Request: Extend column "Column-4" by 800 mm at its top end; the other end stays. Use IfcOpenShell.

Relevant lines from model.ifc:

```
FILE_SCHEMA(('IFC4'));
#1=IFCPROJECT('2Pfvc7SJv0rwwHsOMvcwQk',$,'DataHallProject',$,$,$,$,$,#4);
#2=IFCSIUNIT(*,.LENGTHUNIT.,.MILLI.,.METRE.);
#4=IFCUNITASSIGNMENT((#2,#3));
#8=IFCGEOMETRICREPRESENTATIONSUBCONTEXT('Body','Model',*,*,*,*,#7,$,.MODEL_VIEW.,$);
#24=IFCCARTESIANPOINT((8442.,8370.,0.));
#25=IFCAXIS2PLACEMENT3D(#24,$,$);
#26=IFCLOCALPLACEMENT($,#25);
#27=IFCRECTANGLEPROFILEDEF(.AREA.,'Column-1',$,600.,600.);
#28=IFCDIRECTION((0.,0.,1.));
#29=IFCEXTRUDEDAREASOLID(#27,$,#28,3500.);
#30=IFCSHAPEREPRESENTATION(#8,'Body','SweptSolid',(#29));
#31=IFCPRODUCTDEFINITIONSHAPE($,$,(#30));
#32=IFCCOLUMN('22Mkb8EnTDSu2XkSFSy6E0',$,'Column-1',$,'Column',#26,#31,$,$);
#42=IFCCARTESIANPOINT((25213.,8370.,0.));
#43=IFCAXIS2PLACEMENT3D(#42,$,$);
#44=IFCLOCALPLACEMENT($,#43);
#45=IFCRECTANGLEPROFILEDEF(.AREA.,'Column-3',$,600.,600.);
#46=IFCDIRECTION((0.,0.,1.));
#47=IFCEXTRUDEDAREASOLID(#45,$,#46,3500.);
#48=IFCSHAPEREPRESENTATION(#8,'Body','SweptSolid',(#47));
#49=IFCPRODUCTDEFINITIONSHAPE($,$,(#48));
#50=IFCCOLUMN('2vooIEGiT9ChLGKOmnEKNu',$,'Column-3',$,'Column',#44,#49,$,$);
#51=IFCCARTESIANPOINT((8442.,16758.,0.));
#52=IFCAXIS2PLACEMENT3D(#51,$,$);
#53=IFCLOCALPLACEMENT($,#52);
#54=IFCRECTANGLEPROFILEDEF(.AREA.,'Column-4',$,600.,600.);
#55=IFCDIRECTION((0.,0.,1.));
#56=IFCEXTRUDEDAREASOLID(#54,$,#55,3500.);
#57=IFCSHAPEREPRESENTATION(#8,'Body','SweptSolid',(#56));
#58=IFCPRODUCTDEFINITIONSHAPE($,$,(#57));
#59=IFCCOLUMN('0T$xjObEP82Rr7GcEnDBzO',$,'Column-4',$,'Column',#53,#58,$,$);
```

```python
import ifcopenshell
import ifcopenshell.util.representation
import ifcopenshell.util.unit

model = ifcopenshell.open("model.ifc")
unit_scale = ifcopenshell.util.unit.calculate_unit_scale(model)

member = model.by_guid("0T$xjObEP82Rr7GcEnDBzO")
change = 0.8 / unit_scale

# The extrusion runs towards the end named, so only its depth changes.
body = ifcopenshell.util.representation.get_representation(member, "Model", "Body")
solid = body.Items[0]
old_length = solid.Depth
solid.Depth += change

print(f"length {old_length:g} -> {solid.Depth:g}")

model.write("model-out.ifc")
```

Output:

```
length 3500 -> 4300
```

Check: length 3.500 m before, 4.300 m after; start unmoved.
